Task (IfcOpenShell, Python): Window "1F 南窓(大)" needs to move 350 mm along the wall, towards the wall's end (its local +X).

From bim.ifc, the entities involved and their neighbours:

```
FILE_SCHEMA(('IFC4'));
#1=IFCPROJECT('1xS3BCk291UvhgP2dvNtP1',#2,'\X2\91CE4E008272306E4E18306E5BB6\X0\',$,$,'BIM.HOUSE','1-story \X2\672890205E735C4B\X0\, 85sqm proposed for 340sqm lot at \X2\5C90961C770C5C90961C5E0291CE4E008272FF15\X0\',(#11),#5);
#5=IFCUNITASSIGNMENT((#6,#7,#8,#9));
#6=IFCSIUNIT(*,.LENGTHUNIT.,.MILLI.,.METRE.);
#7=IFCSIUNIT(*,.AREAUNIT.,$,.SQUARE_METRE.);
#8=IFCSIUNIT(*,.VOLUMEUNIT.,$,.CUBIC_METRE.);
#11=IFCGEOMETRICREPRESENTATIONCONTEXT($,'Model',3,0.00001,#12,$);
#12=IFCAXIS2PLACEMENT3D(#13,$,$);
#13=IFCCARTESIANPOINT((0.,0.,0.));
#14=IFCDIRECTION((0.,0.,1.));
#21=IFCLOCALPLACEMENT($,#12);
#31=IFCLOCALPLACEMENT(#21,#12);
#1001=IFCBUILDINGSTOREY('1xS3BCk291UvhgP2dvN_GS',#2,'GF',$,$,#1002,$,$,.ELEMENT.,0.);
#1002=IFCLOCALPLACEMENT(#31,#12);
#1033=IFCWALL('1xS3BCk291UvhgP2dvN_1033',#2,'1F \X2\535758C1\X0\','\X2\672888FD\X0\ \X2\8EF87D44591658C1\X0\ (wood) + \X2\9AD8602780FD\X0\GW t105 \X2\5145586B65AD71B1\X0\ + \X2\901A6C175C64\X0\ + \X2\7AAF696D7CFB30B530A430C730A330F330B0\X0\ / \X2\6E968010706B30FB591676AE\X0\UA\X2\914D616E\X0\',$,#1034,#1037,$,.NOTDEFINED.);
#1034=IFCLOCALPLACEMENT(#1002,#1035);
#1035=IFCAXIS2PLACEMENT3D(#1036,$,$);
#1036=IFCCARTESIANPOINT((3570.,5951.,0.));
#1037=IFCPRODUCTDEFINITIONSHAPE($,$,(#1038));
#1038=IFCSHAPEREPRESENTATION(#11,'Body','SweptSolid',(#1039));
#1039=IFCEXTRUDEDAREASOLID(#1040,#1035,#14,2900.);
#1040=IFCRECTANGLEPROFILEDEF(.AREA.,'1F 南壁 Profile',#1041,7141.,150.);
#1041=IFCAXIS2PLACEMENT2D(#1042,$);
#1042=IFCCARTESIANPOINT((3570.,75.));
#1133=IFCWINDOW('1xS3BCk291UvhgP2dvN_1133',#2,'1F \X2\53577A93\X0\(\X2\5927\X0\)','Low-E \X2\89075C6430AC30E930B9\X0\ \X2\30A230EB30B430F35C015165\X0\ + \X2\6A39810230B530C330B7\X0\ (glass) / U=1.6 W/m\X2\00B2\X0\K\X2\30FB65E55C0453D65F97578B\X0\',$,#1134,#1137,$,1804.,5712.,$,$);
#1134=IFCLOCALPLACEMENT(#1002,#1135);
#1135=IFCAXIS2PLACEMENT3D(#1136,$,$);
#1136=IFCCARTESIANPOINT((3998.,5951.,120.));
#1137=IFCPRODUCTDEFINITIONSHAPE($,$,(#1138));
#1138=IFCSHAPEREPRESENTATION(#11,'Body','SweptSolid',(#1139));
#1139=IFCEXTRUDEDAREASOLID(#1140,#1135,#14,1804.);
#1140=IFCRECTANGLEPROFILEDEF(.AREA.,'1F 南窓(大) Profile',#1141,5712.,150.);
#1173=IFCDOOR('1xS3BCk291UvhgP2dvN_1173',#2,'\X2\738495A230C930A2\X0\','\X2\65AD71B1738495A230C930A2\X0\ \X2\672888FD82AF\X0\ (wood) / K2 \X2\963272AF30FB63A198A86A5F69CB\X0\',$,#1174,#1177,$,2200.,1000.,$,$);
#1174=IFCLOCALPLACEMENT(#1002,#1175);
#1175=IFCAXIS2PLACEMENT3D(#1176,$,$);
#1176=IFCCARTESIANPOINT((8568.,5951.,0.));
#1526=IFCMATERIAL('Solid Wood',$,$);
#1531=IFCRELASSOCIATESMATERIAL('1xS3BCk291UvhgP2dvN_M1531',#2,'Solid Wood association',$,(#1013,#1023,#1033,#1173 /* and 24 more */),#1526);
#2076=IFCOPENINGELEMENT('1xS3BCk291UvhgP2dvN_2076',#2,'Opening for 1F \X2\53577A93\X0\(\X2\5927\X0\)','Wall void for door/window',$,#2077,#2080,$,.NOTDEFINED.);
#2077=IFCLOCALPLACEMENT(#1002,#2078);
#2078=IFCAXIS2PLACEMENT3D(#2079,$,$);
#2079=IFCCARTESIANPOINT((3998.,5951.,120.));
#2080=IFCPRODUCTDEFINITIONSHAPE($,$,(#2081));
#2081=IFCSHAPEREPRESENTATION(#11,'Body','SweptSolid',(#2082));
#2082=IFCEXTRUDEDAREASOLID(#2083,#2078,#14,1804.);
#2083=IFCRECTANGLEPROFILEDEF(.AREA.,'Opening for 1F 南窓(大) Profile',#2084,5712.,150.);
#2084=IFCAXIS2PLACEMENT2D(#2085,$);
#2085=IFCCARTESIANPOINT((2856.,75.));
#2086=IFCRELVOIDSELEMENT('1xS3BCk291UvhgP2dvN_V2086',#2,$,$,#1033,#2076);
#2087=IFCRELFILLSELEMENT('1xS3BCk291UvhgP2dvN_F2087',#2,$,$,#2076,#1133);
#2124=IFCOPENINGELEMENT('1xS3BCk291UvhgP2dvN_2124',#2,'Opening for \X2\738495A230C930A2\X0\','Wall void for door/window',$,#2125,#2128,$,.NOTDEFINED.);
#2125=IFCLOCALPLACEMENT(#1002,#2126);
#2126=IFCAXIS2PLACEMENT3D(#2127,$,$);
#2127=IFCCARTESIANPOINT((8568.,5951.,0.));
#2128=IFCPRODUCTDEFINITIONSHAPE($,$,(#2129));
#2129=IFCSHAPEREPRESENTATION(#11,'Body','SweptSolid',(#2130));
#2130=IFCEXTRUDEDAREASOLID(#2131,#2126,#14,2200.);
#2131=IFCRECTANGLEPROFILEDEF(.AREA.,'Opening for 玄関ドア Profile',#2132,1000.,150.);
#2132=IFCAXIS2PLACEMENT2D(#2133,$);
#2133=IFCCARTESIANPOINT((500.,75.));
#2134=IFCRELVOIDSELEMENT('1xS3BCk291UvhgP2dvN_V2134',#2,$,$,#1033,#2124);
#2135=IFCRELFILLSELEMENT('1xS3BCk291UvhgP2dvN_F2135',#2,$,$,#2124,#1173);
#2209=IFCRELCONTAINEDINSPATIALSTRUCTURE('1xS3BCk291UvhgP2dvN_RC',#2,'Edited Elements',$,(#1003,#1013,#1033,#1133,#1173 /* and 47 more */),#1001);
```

```python
import ifcopenshell
import ifcopenshell.api.geometry
import ifcopenshell.util.placement
import ifcopenshell.util.unit

model = ifcopenshell.open("bim.ifc")
unit_scale = ifcopenshell.util.unit.calculate_unit_scale(model)

window = model.by_id(1133)
opening = window.FillsVoids[0].RelatingOpeningElement
wall = opening.VoidsElements[0].RelatingBuildingElement

wall_matrix = ifcopenshell.util.placement.get_local_placement(wall.ObjectPlacement)
shift = wall_matrix[:3, 0] * 0.35 / unit_scale
before = ifcopenshell.util.placement.get_local_placement(window.ObjectPlacement)[:3, 3].copy()

# The window is not placed relative to its opening, so move both.
for product in (opening, window):
    matrix = ifcopenshell.util.placement.get_local_placement(product.ObjectPlacement)
    matrix[:3, 3] += shift
    ifcopenshell.api.geometry.edit_object_placement(model, product=product, matrix=matrix, is_si=False)

after = ifcopenshell.util.placement.get_local_placement(window.ObjectPlacement)[:3, 3]
print("window moved by", (after - before).round(3) + 0.0)

model.write("bim_rev.ifc")
```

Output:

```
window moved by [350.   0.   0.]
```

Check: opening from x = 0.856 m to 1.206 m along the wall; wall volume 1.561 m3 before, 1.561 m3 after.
